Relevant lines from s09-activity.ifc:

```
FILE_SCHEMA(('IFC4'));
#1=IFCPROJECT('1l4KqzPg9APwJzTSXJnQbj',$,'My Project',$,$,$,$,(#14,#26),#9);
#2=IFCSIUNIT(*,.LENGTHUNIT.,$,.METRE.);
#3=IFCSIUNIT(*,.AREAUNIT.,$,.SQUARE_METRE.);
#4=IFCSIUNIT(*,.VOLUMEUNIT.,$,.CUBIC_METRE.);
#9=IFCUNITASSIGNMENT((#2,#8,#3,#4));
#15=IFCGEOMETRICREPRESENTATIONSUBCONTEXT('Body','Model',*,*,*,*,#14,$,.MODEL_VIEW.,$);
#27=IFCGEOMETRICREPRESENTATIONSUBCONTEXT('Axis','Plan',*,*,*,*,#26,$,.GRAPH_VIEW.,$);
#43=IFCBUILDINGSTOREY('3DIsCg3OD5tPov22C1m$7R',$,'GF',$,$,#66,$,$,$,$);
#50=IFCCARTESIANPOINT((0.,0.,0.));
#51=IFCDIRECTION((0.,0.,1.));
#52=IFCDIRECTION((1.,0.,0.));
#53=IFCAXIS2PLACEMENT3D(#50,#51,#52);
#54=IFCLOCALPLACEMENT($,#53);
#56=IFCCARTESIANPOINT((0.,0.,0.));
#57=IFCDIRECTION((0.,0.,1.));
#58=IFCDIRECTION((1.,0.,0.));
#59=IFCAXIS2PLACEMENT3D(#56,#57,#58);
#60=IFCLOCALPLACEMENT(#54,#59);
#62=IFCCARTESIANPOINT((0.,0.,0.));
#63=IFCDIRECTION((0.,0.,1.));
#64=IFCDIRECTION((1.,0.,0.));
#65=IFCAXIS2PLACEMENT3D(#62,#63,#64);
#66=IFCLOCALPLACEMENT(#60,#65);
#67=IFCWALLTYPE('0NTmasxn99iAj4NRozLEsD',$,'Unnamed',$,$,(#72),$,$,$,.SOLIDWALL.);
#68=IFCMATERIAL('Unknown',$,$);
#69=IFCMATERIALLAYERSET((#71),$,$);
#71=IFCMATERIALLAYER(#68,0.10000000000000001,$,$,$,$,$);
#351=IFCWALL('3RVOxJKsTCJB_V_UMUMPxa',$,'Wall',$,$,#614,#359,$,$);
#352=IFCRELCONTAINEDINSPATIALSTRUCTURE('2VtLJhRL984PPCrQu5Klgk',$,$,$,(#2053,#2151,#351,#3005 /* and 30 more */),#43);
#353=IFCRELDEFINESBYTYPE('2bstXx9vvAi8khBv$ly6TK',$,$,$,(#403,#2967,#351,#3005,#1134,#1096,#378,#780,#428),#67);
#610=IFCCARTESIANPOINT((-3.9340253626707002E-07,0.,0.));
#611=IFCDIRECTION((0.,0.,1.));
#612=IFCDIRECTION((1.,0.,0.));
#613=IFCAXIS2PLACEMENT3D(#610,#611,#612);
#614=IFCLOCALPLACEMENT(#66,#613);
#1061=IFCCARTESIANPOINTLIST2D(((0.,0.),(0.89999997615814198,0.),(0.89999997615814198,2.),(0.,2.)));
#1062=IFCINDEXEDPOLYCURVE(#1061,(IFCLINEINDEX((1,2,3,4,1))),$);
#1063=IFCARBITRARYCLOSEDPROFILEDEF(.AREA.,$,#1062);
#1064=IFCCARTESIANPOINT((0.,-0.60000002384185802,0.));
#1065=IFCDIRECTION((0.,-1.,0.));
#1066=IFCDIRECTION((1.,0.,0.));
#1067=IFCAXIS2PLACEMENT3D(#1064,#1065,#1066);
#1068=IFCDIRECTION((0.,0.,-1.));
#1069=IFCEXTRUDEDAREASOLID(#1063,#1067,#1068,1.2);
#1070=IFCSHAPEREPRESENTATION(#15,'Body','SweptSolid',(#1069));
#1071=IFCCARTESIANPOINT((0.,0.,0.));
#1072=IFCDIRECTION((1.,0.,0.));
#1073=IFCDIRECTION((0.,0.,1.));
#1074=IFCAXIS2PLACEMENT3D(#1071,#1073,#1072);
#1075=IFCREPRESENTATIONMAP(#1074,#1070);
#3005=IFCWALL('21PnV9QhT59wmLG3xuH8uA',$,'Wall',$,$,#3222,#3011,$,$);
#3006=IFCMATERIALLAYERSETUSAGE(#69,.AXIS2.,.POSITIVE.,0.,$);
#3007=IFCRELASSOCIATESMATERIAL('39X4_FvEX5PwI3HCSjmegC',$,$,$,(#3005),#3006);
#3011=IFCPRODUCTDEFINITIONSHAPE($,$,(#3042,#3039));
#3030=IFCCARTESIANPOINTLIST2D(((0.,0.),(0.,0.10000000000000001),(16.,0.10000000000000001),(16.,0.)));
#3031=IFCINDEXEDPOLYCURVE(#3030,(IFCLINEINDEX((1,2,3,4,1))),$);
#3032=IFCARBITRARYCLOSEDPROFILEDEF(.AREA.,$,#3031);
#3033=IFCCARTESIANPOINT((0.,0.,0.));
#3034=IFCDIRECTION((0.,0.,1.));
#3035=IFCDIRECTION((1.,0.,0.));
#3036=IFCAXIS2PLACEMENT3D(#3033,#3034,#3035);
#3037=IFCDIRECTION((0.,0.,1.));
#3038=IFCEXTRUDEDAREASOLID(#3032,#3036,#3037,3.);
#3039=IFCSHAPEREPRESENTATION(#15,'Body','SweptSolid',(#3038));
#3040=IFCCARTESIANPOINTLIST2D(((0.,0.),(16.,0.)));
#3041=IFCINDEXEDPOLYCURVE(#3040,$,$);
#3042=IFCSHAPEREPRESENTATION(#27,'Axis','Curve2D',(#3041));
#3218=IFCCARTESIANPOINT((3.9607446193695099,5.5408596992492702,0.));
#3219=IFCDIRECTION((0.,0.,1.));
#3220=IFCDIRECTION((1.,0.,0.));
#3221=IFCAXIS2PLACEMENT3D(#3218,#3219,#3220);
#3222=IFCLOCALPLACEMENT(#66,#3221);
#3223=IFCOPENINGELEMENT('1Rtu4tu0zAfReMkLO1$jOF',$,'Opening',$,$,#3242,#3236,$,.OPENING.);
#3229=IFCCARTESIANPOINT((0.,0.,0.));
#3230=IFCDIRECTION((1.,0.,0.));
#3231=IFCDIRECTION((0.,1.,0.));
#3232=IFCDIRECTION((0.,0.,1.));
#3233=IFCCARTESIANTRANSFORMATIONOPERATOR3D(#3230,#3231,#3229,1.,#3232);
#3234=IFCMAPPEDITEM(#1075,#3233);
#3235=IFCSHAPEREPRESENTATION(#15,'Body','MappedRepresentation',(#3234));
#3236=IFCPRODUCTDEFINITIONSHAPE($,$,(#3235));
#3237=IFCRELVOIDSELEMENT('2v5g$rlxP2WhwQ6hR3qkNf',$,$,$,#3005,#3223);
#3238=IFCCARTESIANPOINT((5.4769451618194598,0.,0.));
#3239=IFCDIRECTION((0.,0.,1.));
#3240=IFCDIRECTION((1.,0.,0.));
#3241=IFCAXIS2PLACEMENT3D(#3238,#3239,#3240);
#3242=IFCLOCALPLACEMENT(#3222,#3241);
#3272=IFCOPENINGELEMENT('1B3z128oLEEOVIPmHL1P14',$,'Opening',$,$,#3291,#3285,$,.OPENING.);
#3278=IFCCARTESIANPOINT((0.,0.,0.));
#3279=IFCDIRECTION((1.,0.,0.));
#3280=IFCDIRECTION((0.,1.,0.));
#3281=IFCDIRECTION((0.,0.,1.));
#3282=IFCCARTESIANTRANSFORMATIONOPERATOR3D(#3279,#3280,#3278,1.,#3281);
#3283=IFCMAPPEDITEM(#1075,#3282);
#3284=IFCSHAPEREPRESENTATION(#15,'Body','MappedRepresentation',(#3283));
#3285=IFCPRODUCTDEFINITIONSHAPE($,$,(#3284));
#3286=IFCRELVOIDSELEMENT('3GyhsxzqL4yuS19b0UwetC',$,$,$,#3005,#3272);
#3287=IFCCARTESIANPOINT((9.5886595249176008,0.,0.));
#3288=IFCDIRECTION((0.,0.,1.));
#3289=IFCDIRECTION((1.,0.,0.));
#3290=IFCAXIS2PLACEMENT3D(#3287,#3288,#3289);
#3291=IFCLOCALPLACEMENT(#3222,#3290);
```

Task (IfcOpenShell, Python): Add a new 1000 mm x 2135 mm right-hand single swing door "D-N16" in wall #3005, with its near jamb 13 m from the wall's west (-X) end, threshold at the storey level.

```python
import numpy as np
import ifcopenshell
import ifcopenshell.api.feature
import ifcopenshell.api.geometry
import ifcopenshell.api.root
import ifcopenshell.api.spatial
import ifcopenshell.geom
import ifcopenshell.util.element
import ifcopenshell.util.placement
import ifcopenshell.util.representation
import ifcopenshell.util.shape
import ifcopenshell.util.unit

model = ifcopenshell.open("s09-activity.ifc")
unit_scale = ifcopenshell.util.unit.calculate_unit_scale(model)
settings = ifcopenshell.geom.settings()


def volume(element):
    """Net volume in cubic metres, openings subtracted."""
    shape = ifcopenshell.geom.create_shape(settings, element)
    return ifcopenshell.util.shape.get_volume(shape.geometry)


wall = model.by_id(3005)
storey = ifcopenshell.util.element.get_container(wall, ifc_class="IfcBuildingStorey")
context = ifcopenshell.util.representation.get_context(model, "Model", "Body", "MODEL_VIEW")
before = volume(wall)

width, height, from_end, sill = 1, 2.135, 13, 0.0  # metres

# The wall runs along its own X axis, and the end named is its -X end.
wall_shape = ifcopenshell.geom.create_shape(settings, wall)
x, y, z = ifcopenshell.util.shape.get_vertices(wall_shape.geometry).T
start = x.min() + from_end
face, thickness = float(y.min()), float(y.max() - y.min())
wall_matrix = ifcopenshell.util.placement.get_local_placement(wall.ObjectPlacement)
level = ifcopenshell.util.placement.get_local_placement(storey.ObjectPlacement)[2, 3]


def in_wall(x, y):
    """Placement at x, y metres in the wall's axes, at sill height."""
    matrix = wall_matrix.copy()
    matrix[:, 3] = wall_matrix @ np.array([x / unit_scale, y / unit_scale, 0.0, 1.0])
    matrix[2, 3] = level + sill / unit_scale
    return matrix


# Opening: a box that overshoots both wall faces by 50 mm.
opening = ifcopenshell.api.root.create_entity(model, ifc_class="IfcOpeningElement", predefined_type="OPENING")
box = ifcopenshell.api.geometry.add_wall_representation(
    model, context=context, length=width, height=height, thickness=thickness + 0.1
)
ifcopenshell.api.geometry.assign_representation(model, product=opening, representation=box)
ifcopenshell.api.geometry.edit_object_placement(model, product=opening, matrix=in_wall(start, face - 0.05), is_si=False)
ifcopenshell.api.feature.add_feature(model, feature=opening, element=wall)

door = ifcopenshell.api.root.create_entity(model, ifc_class="IfcDoor", name="D-N16", predefined_type="DOOR")
door.OverallWidth, door.OverallHeight = width / unit_scale, height / unit_scale
door.OperationType = "SINGLE_SWING_RIGHT"
body = ifcopenshell.api.geometry.add_door_representation(
    model,
    context=context,
    overall_width=door.OverallWidth,
    overall_height=door.OverallHeight,
    operation_type="SINGLE_SWING_RIGHT",
    lining_properties={"LiningDepth": thickness / unit_scale, "ThresholdDepth": thickness / unit_scale},
)
ifcopenshell.api.geometry.assign_representation(model, product=door, representation=body)
ifcopenshell.api.spatial.assign_container(model, products=[door], relating_structure=storey)
ifcopenshell.api.feature.add_filling(model, opening=opening, element=door)

# The lining spans the wall, so the door starts at the wall face.
ifcopenshell.api.geometry.edit_object_placement(model, product=door, matrix=in_wall(start, face), is_si=False)

after = volume(wall)

print(f"wall volume {before:.3f} -> {after:.3f} m3")

model.write("s09-activity_v2.ifc")
```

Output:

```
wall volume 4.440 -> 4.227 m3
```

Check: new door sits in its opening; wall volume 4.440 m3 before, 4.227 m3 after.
